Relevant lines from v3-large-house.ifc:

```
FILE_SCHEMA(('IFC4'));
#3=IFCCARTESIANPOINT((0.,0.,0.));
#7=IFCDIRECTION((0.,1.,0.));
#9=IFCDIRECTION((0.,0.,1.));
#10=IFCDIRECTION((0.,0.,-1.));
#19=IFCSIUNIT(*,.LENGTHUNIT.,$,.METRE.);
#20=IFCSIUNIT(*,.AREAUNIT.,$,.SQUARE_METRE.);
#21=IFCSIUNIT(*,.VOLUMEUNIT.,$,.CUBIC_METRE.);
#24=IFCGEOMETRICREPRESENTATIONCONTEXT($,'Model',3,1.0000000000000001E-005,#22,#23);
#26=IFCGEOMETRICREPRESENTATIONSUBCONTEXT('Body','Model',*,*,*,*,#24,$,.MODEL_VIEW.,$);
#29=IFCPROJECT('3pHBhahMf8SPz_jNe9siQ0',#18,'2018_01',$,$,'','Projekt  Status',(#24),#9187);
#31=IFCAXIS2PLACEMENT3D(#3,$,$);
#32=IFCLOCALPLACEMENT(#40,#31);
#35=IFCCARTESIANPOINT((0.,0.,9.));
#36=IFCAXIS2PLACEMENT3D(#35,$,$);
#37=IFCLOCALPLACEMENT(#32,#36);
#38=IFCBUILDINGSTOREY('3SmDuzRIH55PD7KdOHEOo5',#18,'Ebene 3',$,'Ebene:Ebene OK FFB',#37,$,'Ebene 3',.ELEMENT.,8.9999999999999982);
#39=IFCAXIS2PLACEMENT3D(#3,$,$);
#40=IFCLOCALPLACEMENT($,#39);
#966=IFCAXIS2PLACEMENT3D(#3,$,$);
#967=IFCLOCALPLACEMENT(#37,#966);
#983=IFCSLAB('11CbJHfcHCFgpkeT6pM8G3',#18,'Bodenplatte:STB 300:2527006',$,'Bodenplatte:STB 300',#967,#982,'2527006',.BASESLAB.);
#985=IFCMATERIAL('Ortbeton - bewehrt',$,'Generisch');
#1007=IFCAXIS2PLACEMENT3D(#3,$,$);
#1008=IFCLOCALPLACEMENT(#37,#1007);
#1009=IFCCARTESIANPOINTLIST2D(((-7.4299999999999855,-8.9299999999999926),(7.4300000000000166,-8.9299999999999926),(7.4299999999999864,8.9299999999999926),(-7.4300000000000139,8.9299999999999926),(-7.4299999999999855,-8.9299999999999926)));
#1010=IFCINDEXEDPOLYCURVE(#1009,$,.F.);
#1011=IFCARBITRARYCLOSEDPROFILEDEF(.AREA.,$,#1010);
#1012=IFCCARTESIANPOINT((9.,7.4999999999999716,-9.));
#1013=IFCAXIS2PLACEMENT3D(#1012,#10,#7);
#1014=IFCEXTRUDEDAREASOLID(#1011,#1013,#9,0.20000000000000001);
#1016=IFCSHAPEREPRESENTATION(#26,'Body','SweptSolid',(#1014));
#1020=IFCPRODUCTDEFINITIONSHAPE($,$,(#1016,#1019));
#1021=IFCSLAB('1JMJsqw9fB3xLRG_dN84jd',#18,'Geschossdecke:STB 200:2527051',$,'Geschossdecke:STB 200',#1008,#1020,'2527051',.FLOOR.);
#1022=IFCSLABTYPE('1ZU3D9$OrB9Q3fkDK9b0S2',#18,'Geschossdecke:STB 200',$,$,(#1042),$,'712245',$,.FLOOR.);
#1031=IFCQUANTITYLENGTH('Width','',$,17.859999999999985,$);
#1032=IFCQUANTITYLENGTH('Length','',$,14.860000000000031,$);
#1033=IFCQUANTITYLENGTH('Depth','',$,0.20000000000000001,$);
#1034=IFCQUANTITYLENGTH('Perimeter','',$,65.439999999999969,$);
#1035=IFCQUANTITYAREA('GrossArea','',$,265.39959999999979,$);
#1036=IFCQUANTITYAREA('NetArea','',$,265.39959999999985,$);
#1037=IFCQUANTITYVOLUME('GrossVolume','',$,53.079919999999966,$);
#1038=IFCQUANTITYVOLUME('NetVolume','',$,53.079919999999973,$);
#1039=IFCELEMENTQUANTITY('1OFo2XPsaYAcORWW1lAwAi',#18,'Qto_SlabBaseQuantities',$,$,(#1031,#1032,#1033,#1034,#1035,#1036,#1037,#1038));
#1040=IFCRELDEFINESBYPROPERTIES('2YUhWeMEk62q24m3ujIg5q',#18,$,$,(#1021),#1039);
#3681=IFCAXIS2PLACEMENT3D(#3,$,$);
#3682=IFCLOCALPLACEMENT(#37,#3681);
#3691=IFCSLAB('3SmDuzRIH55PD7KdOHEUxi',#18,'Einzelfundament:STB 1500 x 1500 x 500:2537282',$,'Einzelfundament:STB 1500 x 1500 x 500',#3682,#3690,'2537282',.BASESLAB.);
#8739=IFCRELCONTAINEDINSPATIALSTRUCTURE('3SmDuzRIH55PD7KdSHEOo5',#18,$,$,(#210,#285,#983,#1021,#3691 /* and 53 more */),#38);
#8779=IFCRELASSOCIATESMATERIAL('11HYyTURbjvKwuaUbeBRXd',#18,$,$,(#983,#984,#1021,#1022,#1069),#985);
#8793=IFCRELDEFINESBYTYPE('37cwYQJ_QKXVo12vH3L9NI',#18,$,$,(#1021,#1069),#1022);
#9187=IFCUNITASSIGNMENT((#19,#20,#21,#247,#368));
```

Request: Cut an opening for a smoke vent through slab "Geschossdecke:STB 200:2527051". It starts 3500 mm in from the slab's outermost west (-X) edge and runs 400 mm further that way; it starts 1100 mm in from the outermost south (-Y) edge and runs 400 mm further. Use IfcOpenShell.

```python
import numpy as np
import ifcopenshell
import ifcopenshell.api.feature
import ifcopenshell.api.geometry
import ifcopenshell.api.pset
import ifcopenshell.api.root
import ifcopenshell.geom
import ifcopenshell.util.element
import ifcopenshell.util.placement
import ifcopenshell.util.representation
import ifcopenshell.util.shape
import ifcopenshell.util.unit

model = ifcopenshell.open("v3-large-house.ifc")
unit_scale = ifcopenshell.util.unit.calculate_unit_scale(model)
area_scale = ifcopenshell.util.unit.calculate_unit_scale(model, "AREAUNIT")
volume_scale = ifcopenshell.util.unit.calculate_unit_scale(model, "VOLUMEUNIT")
settings = ifcopenshell.geom.settings()


def volume(element):
    """Net volume in cubic metres, openings subtracted."""
    shape = ifcopenshell.geom.create_shape(settings, element)
    return ifcopenshell.util.shape.get_volume(shape.geometry)


slab = model.by_guid("1JMJsqw9fB3xLRG_dN84jd")
before = volume(slab)

# Extent in the slab's own axes, in metres. The edges named are its -X and -Y sides.
slab_shape = ifcopenshell.geom.create_shape(settings, slab)
vertices = ifcopenshell.util.shape.get_vertices(slab_shape.geometry)
x_min, y_min, bottom = vertices.min(axis=0)
top = vertices[:, 2].max()

opening = ifcopenshell.api.root.create_entity(model, ifc_class="IfcOpeningElement", name="Smoke vent opening", predefined_type="OPENING")
context = ifcopenshell.util.representation.get_context(model, "Model", "Body", "MODEL_VIEW")
width, depth = 0.4, 0.4
outline = [(0.0, 0.0), (width, 0.0), (width, depth), (0.0, depth), (0.0, 0.0)]
# Overshoot both faces by 50 mm so the cut is clean.
shape = ifcopenshell.api.geometry.add_slab_representation(
    model, context=context, depth=top - bottom + 0.1, polyline=outline
)
ifcopenshell.api.geometry.assign_representation(model, product=opening, representation=shape)

matrix = ifcopenshell.util.placement.get_local_placement(slab.ObjectPlacement)
matrix[:, 3] = matrix @ np.append(np.array([x_min + 3.5, y_min + 1.1, bottom - 0.05]) / unit_scale, 1.0)
ifcopenshell.api.geometry.edit_object_placement(model, product=opening, matrix=matrix, is_si=False)
ifcopenshell.api.feature.add_feature(model, feature=opening, element=slab)

after = volume(slab)

# Update the slab's stored quantities.
qto = model.by_id(ifcopenshell.util.element.get_pset(slab, "Qto_SlabBaseQuantities", should_inherit=False)["id"])
ifcopenshell.api.pset.edit_qto(model, qto=qto, properties={
    "NetArea": after / (top - bottom) / area_scale,
    "NetVolume": after / volume_scale,
})

print(f"slab volume {before:.3f} -> {after:.3f} m3")

model.write("v3-large-house_v2.ifc")
```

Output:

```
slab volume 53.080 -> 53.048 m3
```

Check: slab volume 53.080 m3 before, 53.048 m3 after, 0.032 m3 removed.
